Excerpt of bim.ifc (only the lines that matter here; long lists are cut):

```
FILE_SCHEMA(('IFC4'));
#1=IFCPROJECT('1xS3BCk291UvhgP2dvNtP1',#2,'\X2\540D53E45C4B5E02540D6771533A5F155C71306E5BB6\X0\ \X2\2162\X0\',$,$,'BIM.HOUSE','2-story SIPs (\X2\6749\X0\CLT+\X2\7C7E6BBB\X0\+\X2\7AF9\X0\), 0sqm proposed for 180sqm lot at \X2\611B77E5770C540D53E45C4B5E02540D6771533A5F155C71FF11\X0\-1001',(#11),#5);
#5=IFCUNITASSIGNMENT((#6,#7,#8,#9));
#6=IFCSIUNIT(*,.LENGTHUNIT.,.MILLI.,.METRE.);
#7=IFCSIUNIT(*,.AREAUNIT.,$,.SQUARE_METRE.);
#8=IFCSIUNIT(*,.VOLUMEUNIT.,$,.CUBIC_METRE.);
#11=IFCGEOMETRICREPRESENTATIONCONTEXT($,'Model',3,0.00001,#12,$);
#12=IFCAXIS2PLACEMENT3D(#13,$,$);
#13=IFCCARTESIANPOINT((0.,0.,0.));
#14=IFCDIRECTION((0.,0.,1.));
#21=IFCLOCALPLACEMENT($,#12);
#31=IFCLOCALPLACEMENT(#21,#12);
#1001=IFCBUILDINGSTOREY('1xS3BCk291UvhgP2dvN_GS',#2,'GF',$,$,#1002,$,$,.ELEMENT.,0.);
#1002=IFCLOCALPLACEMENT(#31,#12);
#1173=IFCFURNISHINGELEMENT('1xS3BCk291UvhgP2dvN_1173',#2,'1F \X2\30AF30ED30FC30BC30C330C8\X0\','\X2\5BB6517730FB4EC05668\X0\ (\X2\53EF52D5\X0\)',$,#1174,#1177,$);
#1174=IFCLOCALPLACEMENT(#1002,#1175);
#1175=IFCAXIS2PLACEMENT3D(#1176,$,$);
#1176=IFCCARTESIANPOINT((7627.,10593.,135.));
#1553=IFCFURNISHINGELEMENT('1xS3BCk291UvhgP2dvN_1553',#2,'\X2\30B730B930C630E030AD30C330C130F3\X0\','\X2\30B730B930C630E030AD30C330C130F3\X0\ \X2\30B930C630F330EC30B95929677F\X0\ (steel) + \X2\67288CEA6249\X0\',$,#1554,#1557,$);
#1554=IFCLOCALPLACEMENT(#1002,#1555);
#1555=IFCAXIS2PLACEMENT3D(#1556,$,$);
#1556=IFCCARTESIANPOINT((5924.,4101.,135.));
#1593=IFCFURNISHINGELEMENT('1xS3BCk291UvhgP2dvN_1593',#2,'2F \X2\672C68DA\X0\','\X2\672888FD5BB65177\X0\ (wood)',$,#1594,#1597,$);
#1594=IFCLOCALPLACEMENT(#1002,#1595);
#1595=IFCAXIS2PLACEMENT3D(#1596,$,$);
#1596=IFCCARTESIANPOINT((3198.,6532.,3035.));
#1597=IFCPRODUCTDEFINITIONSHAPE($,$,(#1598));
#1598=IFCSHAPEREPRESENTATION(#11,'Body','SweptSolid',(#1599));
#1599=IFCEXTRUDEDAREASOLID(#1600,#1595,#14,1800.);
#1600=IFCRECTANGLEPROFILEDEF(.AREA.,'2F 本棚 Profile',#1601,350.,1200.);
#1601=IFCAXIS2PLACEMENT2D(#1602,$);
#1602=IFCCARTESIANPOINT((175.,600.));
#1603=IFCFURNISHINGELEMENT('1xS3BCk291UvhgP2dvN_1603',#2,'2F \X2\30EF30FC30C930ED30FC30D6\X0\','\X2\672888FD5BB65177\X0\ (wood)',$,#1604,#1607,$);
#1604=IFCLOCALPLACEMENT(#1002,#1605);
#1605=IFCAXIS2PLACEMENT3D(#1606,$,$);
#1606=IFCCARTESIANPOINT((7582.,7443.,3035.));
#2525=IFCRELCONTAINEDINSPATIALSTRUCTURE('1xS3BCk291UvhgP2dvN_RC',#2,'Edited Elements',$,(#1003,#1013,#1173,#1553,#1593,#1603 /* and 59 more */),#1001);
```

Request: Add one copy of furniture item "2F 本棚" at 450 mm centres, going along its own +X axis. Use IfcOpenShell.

```python
import ifcopenshell
import ifcopenshell.api.geometry
import ifcopenshell.api.root
import ifcopenshell.util.element
import ifcopenshell.util.placement

model = ifcopenshell.open("bim.ifc")


def reuse_history(source, copy):
    """copy_class also copies each property set's owner history, people and application; keep the originals."""
    for rel in copy.IsDefinedBy:
        if rel.is_a("IfcRelDefinesByProperties") and (history := rel.RelatingPropertyDefinition.OwnerHistory):
            rel.RelatingPropertyDefinition.OwnerHistory = source.OwnerHistory
            ifcopenshell.util.element.remove_deep2(model, history)


source = model.by_guid("1xS3BCk291UvhgP2dvN_1593")
base = ifcopenshell.util.placement.get_local_placement(source.ObjectPlacement)
step = base[:3, 0] * 450.0

for i in range(1, 2):
    copy = ifcopenshell.api.root.copy_class(model, product=source)
    copy.Representation = ifcopenshell.util.element.copy_deep(
        model, source.Representation, exclude=["IfcGeometricRepresentationContext", "IfcRepresentationMap"]
    )
    reuse_history(source, copy)
    matrix = base.copy()
    matrix[:3, 3] += i * step
    print("added at", matrix[:3, 3].round(3) + 0.0)
    ifcopenshell.api.geometry.edit_object_placement(model, product=copy, matrix=matrix, is_si=False)

model.write("bim_v2.ifc")
```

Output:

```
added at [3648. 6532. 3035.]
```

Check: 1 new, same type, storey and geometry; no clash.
